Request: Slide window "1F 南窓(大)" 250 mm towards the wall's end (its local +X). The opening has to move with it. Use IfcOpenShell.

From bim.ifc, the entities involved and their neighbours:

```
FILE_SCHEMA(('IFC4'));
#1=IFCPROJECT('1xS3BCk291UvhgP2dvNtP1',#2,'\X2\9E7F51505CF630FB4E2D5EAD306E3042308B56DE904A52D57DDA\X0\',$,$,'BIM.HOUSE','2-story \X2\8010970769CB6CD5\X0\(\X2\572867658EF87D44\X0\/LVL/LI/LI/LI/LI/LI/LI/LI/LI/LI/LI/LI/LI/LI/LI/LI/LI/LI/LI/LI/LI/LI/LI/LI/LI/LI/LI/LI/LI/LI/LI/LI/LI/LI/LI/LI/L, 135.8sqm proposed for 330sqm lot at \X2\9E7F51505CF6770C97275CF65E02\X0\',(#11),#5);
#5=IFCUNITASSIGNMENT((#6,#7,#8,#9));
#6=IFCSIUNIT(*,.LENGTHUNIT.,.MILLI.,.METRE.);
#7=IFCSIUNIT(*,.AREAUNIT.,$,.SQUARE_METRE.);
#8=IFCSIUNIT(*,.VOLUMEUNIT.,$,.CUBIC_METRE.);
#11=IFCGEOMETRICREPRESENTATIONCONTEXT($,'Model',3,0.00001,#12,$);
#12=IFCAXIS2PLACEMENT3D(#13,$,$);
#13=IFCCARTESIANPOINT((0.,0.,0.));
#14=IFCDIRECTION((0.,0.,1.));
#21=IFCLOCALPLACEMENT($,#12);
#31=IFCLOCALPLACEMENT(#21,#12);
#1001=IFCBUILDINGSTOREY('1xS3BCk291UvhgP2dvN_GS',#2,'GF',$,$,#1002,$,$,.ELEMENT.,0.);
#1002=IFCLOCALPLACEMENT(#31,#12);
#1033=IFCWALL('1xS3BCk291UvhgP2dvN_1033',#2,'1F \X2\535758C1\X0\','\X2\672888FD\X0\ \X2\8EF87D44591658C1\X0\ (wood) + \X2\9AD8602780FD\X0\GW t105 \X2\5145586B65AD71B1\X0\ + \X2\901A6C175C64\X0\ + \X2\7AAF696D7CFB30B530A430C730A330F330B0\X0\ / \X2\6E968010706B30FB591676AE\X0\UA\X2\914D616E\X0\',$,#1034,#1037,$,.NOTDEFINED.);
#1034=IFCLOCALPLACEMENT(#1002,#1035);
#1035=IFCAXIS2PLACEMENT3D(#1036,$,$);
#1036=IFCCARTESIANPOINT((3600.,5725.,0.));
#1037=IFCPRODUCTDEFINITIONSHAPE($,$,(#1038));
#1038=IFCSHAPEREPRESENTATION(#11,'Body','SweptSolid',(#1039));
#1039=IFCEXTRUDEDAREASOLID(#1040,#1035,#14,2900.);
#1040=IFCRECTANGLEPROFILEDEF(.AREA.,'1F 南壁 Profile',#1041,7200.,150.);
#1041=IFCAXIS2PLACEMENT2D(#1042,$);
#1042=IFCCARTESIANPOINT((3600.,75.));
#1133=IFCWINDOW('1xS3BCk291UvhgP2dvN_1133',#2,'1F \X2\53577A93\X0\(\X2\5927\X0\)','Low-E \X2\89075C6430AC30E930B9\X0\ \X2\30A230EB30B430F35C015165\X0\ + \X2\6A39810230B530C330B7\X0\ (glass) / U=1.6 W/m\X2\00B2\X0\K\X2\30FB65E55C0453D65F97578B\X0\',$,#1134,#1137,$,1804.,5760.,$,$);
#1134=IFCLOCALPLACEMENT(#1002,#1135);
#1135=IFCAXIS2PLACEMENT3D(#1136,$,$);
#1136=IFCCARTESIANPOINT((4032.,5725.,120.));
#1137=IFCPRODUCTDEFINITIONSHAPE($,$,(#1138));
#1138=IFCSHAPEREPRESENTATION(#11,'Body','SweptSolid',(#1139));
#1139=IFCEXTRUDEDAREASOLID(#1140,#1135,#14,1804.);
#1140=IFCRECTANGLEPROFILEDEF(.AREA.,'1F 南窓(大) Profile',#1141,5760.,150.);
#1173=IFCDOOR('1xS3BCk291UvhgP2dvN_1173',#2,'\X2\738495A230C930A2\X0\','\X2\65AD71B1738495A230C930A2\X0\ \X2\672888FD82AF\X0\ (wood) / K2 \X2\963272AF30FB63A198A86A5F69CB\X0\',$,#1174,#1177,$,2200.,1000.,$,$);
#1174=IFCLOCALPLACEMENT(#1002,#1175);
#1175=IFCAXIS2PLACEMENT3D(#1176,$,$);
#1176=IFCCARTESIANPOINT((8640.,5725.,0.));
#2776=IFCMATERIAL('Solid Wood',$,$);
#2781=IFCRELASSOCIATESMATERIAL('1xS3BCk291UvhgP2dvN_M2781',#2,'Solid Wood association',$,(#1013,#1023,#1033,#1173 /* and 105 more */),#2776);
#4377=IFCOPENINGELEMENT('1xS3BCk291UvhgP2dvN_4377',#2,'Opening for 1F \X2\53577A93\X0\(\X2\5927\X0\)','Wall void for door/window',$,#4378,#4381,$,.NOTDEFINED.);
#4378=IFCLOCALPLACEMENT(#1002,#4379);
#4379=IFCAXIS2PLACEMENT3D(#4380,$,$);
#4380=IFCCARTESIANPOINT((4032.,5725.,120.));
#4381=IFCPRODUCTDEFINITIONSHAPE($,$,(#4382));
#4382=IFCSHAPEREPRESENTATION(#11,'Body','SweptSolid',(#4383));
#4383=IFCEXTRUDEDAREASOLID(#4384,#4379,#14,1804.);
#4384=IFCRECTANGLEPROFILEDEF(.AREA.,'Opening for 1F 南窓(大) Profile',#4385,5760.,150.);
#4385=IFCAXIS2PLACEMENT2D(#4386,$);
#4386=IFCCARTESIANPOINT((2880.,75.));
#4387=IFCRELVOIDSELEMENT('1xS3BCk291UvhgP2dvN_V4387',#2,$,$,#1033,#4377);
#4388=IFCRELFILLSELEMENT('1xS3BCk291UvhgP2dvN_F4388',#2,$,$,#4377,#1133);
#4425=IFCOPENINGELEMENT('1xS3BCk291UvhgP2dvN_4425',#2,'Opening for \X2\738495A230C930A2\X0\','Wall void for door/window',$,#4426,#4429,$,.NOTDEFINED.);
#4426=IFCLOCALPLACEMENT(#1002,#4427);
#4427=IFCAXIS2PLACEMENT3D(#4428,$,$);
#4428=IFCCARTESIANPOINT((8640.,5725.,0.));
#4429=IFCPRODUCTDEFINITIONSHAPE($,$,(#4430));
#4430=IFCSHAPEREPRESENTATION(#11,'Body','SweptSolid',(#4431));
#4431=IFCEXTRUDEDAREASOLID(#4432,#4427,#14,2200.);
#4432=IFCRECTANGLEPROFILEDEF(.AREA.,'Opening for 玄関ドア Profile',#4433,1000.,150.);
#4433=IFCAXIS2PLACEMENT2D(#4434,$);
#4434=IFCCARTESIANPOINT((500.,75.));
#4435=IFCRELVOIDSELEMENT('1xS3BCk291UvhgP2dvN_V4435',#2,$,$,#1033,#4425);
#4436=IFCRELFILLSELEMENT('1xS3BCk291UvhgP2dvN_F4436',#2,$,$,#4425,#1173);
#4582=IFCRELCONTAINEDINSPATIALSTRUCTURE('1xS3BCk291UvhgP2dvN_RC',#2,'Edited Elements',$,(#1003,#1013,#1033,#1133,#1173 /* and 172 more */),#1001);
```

```python
import ifcopenshell
import ifcopenshell.api.geometry
import ifcopenshell.util.placement
import ifcopenshell.util.unit

model = ifcopenshell.open("bim.ifc")
unit_scale = ifcopenshell.util.unit.calculate_unit_scale(model)

window = model.by_id(1133)
opening = window.FillsVoids[0].RelatingOpeningElement
wall = opening.VoidsElements[0].RelatingBuildingElement

wall_matrix = ifcopenshell.util.placement.get_local_placement(wall.ObjectPlacement)
shift = wall_matrix[:3, 0] * 0.25 / unit_scale
before = ifcopenshell.util.placement.get_local_placement(window.ObjectPlacement)[:3, 3].copy()

# The window is not placed relative to its opening, so move both.
for product in (opening, window):
    matrix = ifcopenshell.util.placement.get_local_placement(product.ObjectPlacement)
    matrix[:3, 3] += shift
    ifcopenshell.api.geometry.edit_object_placement(model, product=product, matrix=matrix, is_si=False)

after = ifcopenshell.util.placement.get_local_placement(window.ObjectPlacement)[:3, 3]
print("window moved by", (after - before).round(3) + 0.0)

model.write("bim_updated.ifc")
```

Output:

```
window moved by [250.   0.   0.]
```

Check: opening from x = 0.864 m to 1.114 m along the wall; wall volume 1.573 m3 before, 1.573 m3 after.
